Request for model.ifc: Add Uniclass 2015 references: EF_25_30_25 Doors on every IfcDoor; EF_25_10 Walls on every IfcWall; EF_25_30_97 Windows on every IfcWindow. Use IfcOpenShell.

First a look at what the model holds.

```python
import ifcopenshell

model = ifcopenshell.open("model.ifc")
print(model.schema)
print("classifications:", [c.Name for c in model.by_type("IfcClassification")])
for ifc_class in ("IfcDoor", "IfcRoof", "IfcStair", "IfcWall", "IfcWindow"):
    print(ifc_class, len(model.by_type(ifc_class)))
```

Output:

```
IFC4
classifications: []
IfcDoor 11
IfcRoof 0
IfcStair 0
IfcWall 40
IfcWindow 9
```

```python
import ifcopenshell
import ifcopenshell.api.classification

model = ifcopenshell.open("model.ifc")

system = ifcopenshell.api.classification.add_classification(model, classification="Uniclass 2015")

codes = {
    "IfcDoor": ("EF_25_30_25", "Doors"),
    "IfcWall": ("EF_25_10", "Walls"),
    "IfcWindow": ("EF_25_30_97", "Windows"),
}
for ifc_class, (code, name) in codes.items():
    products = model.by_type(ifc_class)
    ifcopenshell.api.classification.add_reference(
        model, products=products, classification=system, identification=code, name=name
    )
    print(code, len(products))

model.write("model_updated.ifc")
```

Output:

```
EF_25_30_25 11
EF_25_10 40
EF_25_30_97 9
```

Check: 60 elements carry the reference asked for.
